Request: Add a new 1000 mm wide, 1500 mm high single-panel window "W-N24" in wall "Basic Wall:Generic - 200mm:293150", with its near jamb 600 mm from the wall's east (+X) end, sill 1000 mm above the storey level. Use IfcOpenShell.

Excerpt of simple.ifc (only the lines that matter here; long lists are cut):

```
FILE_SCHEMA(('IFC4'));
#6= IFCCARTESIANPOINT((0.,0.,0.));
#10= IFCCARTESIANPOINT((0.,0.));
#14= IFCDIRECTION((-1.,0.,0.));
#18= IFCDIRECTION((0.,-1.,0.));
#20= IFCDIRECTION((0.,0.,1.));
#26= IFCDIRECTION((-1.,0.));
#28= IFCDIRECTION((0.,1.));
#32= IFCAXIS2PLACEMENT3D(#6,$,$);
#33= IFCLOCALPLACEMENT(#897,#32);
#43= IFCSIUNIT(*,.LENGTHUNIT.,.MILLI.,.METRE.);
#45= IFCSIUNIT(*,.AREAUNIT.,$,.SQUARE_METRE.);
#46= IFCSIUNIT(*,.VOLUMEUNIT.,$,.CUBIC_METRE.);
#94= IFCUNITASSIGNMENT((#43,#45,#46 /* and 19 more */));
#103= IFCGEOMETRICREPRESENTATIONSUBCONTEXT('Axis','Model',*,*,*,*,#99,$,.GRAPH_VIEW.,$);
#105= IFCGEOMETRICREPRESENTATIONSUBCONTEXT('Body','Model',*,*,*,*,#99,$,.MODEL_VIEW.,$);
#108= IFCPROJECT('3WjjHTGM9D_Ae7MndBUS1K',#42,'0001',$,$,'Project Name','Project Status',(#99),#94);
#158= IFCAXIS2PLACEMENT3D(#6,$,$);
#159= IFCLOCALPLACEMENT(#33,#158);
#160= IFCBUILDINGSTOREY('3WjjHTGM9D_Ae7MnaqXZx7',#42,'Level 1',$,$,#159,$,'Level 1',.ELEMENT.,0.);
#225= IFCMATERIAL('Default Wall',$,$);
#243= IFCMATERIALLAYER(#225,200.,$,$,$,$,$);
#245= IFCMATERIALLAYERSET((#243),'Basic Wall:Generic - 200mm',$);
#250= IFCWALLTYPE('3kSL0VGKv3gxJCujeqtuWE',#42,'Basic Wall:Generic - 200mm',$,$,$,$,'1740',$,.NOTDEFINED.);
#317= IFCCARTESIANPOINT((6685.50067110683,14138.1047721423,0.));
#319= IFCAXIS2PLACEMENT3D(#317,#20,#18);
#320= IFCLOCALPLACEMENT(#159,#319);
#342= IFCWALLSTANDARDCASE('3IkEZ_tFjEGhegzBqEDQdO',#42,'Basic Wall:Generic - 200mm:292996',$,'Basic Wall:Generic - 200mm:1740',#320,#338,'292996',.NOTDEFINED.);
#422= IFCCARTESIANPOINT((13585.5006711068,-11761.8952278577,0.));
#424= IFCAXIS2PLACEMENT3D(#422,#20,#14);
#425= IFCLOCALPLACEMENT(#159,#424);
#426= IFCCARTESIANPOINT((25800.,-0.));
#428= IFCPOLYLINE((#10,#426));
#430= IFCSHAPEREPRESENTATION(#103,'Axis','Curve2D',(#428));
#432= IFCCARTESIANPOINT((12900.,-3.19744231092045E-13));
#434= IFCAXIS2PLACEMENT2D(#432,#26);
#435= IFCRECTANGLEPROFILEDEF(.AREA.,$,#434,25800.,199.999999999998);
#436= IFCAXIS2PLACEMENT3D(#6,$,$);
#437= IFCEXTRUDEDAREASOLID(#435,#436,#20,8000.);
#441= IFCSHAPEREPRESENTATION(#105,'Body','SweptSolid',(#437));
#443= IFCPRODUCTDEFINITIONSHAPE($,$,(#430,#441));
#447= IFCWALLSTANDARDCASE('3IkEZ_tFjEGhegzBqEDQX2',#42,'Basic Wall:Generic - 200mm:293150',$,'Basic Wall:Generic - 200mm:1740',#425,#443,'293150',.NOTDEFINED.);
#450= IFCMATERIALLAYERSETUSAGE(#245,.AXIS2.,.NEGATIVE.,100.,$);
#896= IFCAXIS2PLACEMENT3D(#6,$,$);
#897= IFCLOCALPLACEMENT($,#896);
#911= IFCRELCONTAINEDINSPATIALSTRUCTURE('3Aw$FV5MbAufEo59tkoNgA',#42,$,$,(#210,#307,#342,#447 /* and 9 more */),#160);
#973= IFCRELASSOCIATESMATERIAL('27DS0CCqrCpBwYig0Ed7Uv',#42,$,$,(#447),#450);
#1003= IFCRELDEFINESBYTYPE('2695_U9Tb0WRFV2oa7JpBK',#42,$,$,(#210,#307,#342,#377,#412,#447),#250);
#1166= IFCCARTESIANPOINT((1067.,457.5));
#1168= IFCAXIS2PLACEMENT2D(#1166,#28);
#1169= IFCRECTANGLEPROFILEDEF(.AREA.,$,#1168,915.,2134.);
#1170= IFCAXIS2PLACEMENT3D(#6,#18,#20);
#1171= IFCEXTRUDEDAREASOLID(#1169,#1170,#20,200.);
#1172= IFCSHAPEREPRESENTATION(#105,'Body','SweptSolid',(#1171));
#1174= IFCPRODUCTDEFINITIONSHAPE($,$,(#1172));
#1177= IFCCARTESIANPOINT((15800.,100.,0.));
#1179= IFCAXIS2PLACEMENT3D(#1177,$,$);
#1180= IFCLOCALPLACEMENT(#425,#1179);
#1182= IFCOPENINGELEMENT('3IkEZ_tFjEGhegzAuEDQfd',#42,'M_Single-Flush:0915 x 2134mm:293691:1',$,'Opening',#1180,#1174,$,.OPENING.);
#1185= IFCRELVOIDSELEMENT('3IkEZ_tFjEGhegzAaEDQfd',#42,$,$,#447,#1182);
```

```python
import numpy as np
import ifcopenshell
import ifcopenshell.api.feature
import ifcopenshell.api.geometry
import ifcopenshell.api.root
import ifcopenshell.api.spatial
import ifcopenshell.geom
import ifcopenshell.util.element
import ifcopenshell.util.placement
import ifcopenshell.util.representation
import ifcopenshell.util.shape
import ifcopenshell.util.unit

model = ifcopenshell.open("simple.ifc")
unit_scale = ifcopenshell.util.unit.calculate_unit_scale(model)
settings = ifcopenshell.geom.settings()


def volume(element):
    """Net volume in cubic metres, openings subtracted."""
    shape = ifcopenshell.geom.create_shape(settings, element)
    return ifcopenshell.util.shape.get_volume(shape.geometry)


wall = model.by_guid("3IkEZ_tFjEGhegzBqEDQX2")
storey = ifcopenshell.util.element.get_container(wall, ifc_class="IfcBuildingStorey")
context = ifcopenshell.util.representation.get_context(model, "Model", "Body", "MODEL_VIEW")
before = volume(wall)

width, height, from_end, sill = 1, 1.5, 0.6, 1  # metres

# The wall runs along its own X axis, and the end named is its -X end.
wall_shape = ifcopenshell.geom.create_shape(settings, wall)
x, y, z = ifcopenshell.util.shape.get_vertices(wall_shape.geometry).T
start = x.min() + from_end
face, thickness = float(y.min()), float(y.max() - y.min())
wall_matrix = ifcopenshell.util.placement.get_local_placement(wall.ObjectPlacement)
level = ifcopenshell.util.placement.get_local_placement(storey.ObjectPlacement)[2, 3]


def in_wall(x, y):
    """Placement at x, y metres in the wall's axes, at sill height."""
    matrix = wall_matrix.copy()
    matrix[:, 3] = wall_matrix @ np.array([x / unit_scale, y / unit_scale, 0.0, 1.0])
    matrix[2, 3] = level + sill / unit_scale
    return matrix


# Opening: a box that overshoots both wall faces by 50 mm.
opening = ifcopenshell.api.root.create_entity(model, ifc_class="IfcOpeningElement", predefined_type="OPENING")
box = ifcopenshell.api.geometry.add_wall_representation(
    model, context=context, length=width, height=height, thickness=thickness + 0.1
)
ifcopenshell.api.geometry.assign_representation(model, product=opening, representation=box)
ifcopenshell.api.geometry.edit_object_placement(model, product=opening, matrix=in_wall(start, face - 0.05), is_si=False)
ifcopenshell.api.feature.add_feature(model, feature=opening, element=wall)

window = ifcopenshell.api.root.create_entity(model, ifc_class="IfcWindow", name="W-N24", predefined_type="WINDOW")
window.OverallWidth, window.OverallHeight = width / unit_scale, height / unit_scale
window.PartitioningType = "SINGLE_PANEL"
body = ifcopenshell.api.geometry.add_window_representation(
    model,
    context=context,
    overall_width=window.OverallWidth,
    overall_height=window.OverallHeight,
    partition_type="SINGLE_PANEL",
)
ifcopenshell.api.geometry.assign_representation(model, product=window, representation=body)
ifcopenshell.api.spatial.assign_container(model, products=[window], relating_structure=storey)
ifcopenshell.api.feature.add_filling(model, opening=opening, element=window)

# Centre the window in the wall's thickness.
ifcopenshell.api.geometry.edit_object_placement(model, product=window, matrix=in_wall(start, face), is_si=False)
window_shape = ifcopenshell.geom.create_shape(settings, window)
depth = ifcopenshell.util.shape.get_vertices(window_shape.geometry)[:, 1]
offset = face + thickness / 2 - (depth.min() + depth.max()) / 2
ifcopenshell.api.geometry.edit_object_placement(model, product=window, matrix=in_wall(start, offset), is_si=False)

after = volume(wall)

print(f"wall volume {before:.3f} -> {after:.3f} m3")

model.write("simple_updated.ifc")
```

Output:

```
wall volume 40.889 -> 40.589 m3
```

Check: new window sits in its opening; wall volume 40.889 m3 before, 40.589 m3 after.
